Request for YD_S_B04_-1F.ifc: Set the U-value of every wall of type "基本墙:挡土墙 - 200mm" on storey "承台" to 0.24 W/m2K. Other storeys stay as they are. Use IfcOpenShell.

First a look at what the model holds.

```python
import ifcopenshell
import ifcopenshell.util.element

model = ifcopenshell.open("YD_S_B04_-1F.ifc")
print(model.schema)
storey = next(s for s in model.by_type("IfcBuildingStorey") if s.Name == "承台")
walls = [e for e in ifcopenshell.util.element.get_decomposition(storey) if e.is_a("IfcWall")]
seen = {}
for e in walls:
    element_type = ifcopenshell.util.element.get_type(e)
    key = (element_type.Name if element_type != e and element_type else None, ifcopenshell.util.element.get_pset(e, "Pset_WallCommon", "ThermalTransmittance"))
    seen[key] = seen.get(key, 0) + 1
for (name, value), count in sorted(seen.items(), key=str):
    print(count, "x", name, "|", value)
```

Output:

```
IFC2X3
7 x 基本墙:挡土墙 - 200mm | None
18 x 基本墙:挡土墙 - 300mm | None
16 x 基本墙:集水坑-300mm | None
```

```python
import ifcopenshell
import ifcopenshell.api.pset
import ifcopenshell.util.element

model = ifcopenshell.open("YD_S_B04_-1F.ifc")

storey = next(s for s in model.by_type("IfcBuildingStorey") if s.Name == "承台")
walls = [e for e in ifcopenshell.util.element.get_decomposition(storey) if e.is_a("IfcWall")]

count = 0
for e in walls:
    element_type = ifcopenshell.util.element.get_type(e)
    if element_type in (None, e) or element_type.Name != "基本墙:挡土墙 - 200mm":
        continue
    # add_pset returns the element's existing set when there is one.
    pset = ifcopenshell.api.pset.add_pset(model, product=e, name="Pset_WallCommon")
    ifcopenshell.api.pset.edit_pset(model, pset=pset, properties={"ThermalTransmittance": 0.24})
    count += 1

print(count, "walls updated")

model.write("YD_S_B04_-1F_v2.ifc")
```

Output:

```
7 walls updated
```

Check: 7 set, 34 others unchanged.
